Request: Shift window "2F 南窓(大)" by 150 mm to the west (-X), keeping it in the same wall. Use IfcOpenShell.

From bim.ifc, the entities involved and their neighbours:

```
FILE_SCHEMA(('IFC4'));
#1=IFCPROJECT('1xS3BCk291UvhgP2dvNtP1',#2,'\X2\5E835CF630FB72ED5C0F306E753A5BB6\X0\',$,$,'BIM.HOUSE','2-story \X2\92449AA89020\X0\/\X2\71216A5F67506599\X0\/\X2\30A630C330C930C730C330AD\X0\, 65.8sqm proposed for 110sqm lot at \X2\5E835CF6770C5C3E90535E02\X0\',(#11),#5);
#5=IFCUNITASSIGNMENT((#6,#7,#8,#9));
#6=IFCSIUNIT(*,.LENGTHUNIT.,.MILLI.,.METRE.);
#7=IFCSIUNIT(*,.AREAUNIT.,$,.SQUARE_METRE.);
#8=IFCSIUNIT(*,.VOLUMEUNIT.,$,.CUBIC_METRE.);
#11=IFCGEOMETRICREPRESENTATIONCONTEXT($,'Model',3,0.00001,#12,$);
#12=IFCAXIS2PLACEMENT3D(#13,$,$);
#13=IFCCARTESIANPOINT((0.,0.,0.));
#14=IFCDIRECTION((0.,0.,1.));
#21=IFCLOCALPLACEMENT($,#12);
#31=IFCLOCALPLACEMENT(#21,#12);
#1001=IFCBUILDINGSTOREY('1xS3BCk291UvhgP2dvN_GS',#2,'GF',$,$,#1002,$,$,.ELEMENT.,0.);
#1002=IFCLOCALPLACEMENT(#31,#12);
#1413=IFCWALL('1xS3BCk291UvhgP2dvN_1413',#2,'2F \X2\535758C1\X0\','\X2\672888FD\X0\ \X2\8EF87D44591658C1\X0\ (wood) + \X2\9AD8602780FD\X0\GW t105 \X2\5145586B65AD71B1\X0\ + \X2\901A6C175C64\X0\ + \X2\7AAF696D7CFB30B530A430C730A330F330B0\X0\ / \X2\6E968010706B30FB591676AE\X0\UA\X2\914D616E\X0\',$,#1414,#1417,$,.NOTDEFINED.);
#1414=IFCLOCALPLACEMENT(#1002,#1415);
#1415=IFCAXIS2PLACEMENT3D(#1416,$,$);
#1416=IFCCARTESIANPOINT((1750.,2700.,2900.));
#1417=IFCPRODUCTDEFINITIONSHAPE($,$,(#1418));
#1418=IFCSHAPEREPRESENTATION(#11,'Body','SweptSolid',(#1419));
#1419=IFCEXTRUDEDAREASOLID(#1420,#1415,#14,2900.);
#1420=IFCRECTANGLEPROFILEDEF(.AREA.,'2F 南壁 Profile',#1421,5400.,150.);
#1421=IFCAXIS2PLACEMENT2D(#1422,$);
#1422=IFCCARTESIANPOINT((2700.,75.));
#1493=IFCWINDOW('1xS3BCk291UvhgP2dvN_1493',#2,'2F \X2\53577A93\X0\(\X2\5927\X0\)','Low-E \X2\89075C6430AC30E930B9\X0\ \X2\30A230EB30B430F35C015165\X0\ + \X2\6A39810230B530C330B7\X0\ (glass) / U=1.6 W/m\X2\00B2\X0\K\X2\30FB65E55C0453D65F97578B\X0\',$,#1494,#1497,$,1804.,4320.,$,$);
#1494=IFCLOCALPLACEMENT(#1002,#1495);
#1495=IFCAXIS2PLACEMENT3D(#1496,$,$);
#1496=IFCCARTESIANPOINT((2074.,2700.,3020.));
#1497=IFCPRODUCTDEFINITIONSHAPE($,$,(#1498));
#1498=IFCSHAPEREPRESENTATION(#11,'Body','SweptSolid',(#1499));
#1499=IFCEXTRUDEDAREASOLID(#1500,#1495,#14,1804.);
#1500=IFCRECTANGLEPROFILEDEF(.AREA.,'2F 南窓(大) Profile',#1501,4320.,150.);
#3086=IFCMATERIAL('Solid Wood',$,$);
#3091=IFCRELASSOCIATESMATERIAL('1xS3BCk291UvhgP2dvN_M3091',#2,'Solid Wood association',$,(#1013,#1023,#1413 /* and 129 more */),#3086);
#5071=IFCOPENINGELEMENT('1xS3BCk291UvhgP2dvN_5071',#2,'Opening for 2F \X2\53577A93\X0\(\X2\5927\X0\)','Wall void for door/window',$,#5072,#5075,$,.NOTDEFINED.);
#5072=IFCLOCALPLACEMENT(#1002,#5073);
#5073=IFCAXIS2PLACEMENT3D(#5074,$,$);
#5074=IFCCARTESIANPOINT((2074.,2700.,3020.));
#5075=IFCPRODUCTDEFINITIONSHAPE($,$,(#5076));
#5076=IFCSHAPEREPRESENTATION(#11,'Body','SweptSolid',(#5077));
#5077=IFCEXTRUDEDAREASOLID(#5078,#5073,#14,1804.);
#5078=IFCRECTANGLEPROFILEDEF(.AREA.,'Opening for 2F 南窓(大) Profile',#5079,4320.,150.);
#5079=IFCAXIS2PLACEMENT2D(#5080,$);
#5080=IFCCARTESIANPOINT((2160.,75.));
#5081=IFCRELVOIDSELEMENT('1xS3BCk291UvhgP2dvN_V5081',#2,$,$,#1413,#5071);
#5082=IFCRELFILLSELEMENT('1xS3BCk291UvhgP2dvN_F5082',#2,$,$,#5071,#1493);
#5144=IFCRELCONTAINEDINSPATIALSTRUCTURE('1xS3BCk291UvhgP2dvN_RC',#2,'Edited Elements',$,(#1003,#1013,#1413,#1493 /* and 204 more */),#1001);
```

```python
import ifcopenshell
import ifcopenshell.api.geometry
import ifcopenshell.util.placement
import ifcopenshell.util.unit

model = ifcopenshell.open("bim.ifc")
unit_scale = ifcopenshell.util.unit.calculate_unit_scale(model)

window = model.by_id(1493)
opening = window.FillsVoids[0].RelatingOpeningElement
wall = opening.VoidsElements[0].RelatingBuildingElement

wall_matrix = ifcopenshell.util.placement.get_local_placement(wall.ObjectPlacement)
shift = wall_matrix[:3, 0] * -0.15 / unit_scale
before = ifcopenshell.util.placement.get_local_placement(window.ObjectPlacement)[:3, 3].copy()

# The window is not placed relative to its opening, so move both.
for product in (opening, window):
    matrix = ifcopenshell.util.placement.get_local_placement(product.ObjectPlacement)
    matrix[:3, 3] += shift
    ifcopenshell.api.geometry.edit_object_placement(model, product=product, matrix=matrix, is_si=False)

after = ifcopenshell.util.placement.get_local_placement(window.ObjectPlacement)[:3, 3]
print("window moved by", (after - before).round(3) + 0.0)

model.write("bim_rev.ifc")
```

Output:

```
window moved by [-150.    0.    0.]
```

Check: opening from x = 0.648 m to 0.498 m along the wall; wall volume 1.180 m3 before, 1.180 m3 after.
